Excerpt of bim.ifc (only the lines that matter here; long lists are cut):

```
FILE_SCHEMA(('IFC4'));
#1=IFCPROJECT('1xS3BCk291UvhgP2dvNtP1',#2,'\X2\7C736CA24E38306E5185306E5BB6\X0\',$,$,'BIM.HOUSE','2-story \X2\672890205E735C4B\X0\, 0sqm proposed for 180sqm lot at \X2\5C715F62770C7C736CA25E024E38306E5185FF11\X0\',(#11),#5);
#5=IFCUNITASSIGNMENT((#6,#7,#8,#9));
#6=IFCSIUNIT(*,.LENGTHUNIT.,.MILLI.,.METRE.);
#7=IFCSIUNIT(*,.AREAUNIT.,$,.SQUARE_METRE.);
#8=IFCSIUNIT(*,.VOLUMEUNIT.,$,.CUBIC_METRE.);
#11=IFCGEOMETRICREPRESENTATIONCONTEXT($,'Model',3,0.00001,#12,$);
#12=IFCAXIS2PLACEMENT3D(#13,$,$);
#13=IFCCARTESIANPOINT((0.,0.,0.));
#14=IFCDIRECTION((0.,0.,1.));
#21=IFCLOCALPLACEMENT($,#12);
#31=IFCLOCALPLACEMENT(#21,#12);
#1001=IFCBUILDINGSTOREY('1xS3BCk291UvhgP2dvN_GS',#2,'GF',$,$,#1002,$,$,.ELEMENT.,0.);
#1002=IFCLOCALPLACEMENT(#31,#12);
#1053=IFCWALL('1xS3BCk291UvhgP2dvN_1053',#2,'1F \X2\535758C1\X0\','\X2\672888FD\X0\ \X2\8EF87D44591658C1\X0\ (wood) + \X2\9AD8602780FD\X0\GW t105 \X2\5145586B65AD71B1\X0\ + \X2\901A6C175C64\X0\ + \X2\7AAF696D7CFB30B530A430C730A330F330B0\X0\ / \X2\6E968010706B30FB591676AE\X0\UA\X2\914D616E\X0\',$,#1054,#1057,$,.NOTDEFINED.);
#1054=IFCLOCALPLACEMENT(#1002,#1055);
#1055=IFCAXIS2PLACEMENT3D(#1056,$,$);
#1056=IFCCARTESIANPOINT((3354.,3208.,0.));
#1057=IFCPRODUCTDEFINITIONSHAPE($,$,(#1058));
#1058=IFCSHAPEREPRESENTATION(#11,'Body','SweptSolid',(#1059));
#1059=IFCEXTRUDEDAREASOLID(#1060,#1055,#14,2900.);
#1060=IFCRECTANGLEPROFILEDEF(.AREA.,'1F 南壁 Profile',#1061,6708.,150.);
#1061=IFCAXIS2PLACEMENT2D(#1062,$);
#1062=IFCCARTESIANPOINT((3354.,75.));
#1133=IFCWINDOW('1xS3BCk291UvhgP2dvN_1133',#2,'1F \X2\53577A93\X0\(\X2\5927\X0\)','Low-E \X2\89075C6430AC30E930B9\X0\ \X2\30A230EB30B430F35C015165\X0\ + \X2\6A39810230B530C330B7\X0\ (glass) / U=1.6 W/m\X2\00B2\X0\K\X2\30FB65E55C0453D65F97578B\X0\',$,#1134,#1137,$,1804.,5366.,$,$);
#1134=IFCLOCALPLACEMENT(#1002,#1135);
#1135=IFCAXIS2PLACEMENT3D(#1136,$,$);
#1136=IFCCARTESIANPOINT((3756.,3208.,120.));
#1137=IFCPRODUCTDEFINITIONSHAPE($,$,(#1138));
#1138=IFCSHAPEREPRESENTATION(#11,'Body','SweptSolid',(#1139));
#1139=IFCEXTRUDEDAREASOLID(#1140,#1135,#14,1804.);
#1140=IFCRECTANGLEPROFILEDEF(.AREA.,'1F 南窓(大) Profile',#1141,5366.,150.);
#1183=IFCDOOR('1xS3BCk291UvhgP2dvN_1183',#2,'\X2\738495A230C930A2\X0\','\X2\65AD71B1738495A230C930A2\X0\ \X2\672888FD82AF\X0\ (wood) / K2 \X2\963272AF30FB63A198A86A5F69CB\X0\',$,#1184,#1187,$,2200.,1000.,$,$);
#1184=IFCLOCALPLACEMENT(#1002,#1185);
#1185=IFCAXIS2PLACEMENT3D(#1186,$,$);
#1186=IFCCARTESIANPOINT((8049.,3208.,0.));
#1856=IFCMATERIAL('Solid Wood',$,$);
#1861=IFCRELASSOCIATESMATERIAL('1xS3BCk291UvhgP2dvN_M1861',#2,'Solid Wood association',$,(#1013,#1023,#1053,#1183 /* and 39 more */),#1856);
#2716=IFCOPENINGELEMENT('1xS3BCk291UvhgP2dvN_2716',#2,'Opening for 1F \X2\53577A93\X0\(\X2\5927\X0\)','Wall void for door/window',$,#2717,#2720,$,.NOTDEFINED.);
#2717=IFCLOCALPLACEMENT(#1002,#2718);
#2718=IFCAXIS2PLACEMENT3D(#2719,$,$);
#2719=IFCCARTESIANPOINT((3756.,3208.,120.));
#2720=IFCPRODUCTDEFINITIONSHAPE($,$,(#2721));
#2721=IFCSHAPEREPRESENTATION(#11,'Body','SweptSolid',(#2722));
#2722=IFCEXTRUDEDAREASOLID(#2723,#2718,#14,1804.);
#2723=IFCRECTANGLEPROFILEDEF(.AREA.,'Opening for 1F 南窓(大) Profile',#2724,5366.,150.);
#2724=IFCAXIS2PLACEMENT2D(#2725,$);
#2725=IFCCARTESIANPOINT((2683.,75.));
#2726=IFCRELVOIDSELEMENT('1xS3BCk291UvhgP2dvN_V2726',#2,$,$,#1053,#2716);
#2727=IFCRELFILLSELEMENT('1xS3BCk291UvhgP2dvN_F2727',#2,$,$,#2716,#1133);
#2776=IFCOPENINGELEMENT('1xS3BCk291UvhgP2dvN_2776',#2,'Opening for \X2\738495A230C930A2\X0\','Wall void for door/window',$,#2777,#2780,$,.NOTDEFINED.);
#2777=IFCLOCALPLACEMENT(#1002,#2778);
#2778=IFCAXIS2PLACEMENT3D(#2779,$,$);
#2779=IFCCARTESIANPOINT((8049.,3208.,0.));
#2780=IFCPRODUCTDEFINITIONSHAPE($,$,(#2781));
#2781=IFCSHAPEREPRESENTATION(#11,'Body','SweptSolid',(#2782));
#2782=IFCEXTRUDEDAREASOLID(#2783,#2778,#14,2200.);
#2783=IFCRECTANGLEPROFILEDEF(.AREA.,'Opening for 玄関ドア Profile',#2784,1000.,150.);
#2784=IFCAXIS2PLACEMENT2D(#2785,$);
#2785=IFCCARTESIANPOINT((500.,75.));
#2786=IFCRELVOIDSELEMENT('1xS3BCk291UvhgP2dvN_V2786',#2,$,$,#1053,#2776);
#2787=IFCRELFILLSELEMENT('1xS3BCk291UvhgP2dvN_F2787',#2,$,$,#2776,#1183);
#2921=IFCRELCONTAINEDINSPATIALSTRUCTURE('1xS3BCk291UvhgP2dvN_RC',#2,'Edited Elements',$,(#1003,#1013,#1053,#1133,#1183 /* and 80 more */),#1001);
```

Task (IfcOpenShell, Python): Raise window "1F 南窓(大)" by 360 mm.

```python
import numpy as np
import ifcopenshell
import ifcopenshell.api.geometry
import ifcopenshell.util.placement
import ifcopenshell.util.unit

model = ifcopenshell.open("bim.ifc")
unit_scale = ifcopenshell.util.unit.calculate_unit_scale(model)

window = model.by_guid("1xS3BCk291UvhgP2dvN_1133")
opening = window.FillsVoids[0].RelatingOpeningElement
dz = 0.36 / unit_scale

shift = np.array([0.0, 0.0, dz])
# The window is not placed relative to its opening, so move both.
for product in (opening, window):
    matrix = ifcopenshell.util.placement.get_local_placement(product.ObjectPlacement)
    matrix[:3, 3] += shift
    ifcopenshell.api.geometry.edit_object_placement(model, product=product, matrix=matrix, is_si=False)

print(f"moved by {dz * unit_scale:+.3f} m")

model.write("bim-out.ifc")
```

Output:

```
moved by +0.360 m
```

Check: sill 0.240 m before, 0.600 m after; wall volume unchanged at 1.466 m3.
